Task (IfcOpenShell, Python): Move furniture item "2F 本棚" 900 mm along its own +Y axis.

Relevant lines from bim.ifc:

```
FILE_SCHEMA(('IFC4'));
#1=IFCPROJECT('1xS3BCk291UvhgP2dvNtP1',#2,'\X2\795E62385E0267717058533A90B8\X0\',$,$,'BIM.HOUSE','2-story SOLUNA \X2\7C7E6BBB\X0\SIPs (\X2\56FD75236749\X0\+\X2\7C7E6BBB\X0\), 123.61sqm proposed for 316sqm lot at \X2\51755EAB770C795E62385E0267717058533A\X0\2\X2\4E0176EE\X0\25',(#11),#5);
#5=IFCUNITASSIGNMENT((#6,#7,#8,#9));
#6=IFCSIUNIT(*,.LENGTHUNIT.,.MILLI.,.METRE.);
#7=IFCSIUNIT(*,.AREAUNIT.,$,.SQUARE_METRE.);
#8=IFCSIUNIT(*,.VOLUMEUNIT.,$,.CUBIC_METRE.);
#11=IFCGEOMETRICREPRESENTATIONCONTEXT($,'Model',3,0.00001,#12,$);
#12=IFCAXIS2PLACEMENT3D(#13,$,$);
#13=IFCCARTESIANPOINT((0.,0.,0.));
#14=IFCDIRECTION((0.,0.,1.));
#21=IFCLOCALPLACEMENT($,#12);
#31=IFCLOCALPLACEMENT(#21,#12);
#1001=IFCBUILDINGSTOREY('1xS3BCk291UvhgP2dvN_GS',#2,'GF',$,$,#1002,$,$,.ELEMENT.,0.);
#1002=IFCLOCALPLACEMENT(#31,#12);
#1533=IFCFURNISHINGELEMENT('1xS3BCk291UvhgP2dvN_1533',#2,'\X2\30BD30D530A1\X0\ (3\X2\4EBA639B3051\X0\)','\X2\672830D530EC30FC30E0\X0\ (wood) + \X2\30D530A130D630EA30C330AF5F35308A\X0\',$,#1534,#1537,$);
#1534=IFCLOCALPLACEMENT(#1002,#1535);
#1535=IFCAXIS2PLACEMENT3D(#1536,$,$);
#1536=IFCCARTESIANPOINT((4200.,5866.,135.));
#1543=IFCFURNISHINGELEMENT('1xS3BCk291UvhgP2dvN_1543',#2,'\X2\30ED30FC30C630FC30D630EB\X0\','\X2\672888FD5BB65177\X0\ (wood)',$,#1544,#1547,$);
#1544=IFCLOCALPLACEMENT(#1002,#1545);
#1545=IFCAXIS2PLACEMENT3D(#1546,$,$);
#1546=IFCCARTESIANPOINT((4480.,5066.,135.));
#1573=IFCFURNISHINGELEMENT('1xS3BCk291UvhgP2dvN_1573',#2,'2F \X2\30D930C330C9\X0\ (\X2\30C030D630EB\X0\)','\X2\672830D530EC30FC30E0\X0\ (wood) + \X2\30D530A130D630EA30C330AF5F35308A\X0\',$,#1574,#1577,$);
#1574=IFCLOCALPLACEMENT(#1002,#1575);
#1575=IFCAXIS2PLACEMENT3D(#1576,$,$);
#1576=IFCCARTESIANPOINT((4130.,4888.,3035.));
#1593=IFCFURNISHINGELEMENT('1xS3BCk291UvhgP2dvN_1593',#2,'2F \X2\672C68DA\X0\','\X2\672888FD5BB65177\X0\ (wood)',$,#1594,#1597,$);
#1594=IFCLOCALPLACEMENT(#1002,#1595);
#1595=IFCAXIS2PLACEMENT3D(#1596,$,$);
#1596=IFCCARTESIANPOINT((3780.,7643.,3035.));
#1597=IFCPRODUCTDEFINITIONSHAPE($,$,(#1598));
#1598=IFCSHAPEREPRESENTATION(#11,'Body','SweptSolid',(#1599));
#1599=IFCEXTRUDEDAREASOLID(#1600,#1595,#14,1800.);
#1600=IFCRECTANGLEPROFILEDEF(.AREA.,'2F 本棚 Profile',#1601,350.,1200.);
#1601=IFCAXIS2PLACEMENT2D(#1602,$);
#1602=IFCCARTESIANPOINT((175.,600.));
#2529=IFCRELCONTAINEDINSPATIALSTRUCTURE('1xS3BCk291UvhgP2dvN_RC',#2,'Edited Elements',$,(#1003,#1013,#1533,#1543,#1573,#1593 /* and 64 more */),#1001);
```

```python
import ifcopenshell
import ifcopenshell.api.geometry
import ifcopenshell.util.placement

model = ifcopenshell.open("bim.ifc")

item = model.by_id(1593)
matrix = ifcopenshell.util.placement.get_local_placement(item.ObjectPlacement)
matrix[:3, 3] += matrix[:3, 1] * 900.0
ifcopenshell.api.geometry.edit_object_placement(model, product=item, matrix=matrix, is_si=False)

print(ifcopenshell.util.placement.get_local_placement(item.ObjectPlacement).round(3) + 0.0)

model.write("bim_rev.ifc")
```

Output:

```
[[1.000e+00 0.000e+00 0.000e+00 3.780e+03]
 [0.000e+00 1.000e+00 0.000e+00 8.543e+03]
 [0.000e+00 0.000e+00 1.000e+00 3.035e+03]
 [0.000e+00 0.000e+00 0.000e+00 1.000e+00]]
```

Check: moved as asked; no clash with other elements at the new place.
